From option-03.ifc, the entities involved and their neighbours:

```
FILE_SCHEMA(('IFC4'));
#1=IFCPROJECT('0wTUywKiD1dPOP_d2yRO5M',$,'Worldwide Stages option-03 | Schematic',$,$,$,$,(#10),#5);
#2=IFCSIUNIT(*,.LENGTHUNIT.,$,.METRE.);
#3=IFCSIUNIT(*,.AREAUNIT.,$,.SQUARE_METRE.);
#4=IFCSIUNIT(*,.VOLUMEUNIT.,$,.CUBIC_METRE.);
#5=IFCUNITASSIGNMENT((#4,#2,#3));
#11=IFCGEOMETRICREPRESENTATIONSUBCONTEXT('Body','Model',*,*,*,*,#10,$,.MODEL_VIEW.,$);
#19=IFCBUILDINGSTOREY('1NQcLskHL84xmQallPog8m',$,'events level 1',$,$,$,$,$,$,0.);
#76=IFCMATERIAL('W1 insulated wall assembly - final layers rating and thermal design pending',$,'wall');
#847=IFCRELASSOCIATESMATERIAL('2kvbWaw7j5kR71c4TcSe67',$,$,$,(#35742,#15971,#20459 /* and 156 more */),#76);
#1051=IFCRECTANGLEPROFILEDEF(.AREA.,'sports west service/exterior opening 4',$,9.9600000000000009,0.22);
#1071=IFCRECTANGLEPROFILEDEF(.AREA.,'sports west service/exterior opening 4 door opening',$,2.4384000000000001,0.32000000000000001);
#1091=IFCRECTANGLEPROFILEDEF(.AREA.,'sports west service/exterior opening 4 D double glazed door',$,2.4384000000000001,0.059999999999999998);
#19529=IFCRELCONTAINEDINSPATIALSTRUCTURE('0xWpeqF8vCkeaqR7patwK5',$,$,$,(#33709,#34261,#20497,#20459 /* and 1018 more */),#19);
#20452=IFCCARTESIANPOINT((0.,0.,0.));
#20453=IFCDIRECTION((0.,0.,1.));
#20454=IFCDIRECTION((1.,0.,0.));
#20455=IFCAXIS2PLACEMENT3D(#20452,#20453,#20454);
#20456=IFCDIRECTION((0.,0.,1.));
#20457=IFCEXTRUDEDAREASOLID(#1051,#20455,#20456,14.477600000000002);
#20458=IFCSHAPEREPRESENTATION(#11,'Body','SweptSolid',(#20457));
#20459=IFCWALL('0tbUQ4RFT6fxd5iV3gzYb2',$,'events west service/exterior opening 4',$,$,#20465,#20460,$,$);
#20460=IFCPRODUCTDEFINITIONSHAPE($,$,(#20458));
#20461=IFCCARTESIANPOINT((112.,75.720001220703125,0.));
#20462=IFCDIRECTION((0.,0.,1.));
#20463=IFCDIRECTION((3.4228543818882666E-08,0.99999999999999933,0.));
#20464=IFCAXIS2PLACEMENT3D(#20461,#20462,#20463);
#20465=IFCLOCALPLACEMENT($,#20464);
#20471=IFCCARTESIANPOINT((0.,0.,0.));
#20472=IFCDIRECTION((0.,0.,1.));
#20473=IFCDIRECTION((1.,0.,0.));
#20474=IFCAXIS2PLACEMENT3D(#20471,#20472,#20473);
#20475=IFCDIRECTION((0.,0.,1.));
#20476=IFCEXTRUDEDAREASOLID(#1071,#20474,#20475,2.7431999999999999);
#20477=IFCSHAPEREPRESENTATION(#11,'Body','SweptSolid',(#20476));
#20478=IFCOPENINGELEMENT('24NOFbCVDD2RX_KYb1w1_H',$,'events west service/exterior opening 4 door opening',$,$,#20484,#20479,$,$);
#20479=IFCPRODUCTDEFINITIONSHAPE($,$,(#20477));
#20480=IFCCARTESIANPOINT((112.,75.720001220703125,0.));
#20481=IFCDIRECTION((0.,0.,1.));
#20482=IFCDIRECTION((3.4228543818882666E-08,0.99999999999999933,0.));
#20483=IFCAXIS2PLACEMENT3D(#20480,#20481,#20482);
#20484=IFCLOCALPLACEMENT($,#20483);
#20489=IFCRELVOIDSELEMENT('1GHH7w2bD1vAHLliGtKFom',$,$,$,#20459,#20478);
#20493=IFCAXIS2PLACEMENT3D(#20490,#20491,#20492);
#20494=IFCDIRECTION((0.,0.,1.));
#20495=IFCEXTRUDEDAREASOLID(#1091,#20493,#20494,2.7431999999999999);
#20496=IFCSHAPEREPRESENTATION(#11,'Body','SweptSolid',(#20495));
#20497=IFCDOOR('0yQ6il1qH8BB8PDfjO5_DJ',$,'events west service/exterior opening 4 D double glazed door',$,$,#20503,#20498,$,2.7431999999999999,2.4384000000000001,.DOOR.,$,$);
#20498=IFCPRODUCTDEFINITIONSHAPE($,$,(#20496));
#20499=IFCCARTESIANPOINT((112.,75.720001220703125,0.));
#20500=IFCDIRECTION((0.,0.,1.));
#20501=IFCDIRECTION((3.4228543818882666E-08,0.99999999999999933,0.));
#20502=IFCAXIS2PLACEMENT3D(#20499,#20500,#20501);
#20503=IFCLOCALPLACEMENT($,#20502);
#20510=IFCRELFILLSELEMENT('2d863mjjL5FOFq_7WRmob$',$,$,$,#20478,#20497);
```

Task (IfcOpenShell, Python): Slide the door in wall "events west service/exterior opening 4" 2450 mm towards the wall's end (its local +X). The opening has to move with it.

```python
import ifcopenshell
import ifcopenshell.api.geometry
import ifcopenshell.util.placement

model = ifcopenshell.open("option-03.ifc")

door = model.by_guid("0yQ6il1qH8BB8PDfjO5_DJ")
opening = door.FillsVoids[0].RelatingOpeningElement
wall = opening.VoidsElements[0].RelatingBuildingElement

wall_matrix = ifcopenshell.util.placement.get_local_placement(wall.ObjectPlacement)
shift = wall_matrix[:3, 0] * 2.45
before = ifcopenshell.util.placement.get_local_placement(door.ObjectPlacement)[:3, 3].copy()

# The door is not placed relative to its opening, so move both.
for product in (opening, door):
    matrix = ifcopenshell.util.placement.get_local_placement(product.ObjectPlacement)
    matrix[:3, 3] += shift
    ifcopenshell.api.geometry.edit_object_placement(model, product=product, matrix=matrix, is_si=False)

after = ifcopenshell.util.placement.get_local_placement(door.ObjectPlacement)[:3, 3]
print("door moved by", (after - before).round(3) + 0.0)

model.write("option-03_v2.ifc")
```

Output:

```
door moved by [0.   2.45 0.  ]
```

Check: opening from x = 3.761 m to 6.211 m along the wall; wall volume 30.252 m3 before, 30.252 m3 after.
